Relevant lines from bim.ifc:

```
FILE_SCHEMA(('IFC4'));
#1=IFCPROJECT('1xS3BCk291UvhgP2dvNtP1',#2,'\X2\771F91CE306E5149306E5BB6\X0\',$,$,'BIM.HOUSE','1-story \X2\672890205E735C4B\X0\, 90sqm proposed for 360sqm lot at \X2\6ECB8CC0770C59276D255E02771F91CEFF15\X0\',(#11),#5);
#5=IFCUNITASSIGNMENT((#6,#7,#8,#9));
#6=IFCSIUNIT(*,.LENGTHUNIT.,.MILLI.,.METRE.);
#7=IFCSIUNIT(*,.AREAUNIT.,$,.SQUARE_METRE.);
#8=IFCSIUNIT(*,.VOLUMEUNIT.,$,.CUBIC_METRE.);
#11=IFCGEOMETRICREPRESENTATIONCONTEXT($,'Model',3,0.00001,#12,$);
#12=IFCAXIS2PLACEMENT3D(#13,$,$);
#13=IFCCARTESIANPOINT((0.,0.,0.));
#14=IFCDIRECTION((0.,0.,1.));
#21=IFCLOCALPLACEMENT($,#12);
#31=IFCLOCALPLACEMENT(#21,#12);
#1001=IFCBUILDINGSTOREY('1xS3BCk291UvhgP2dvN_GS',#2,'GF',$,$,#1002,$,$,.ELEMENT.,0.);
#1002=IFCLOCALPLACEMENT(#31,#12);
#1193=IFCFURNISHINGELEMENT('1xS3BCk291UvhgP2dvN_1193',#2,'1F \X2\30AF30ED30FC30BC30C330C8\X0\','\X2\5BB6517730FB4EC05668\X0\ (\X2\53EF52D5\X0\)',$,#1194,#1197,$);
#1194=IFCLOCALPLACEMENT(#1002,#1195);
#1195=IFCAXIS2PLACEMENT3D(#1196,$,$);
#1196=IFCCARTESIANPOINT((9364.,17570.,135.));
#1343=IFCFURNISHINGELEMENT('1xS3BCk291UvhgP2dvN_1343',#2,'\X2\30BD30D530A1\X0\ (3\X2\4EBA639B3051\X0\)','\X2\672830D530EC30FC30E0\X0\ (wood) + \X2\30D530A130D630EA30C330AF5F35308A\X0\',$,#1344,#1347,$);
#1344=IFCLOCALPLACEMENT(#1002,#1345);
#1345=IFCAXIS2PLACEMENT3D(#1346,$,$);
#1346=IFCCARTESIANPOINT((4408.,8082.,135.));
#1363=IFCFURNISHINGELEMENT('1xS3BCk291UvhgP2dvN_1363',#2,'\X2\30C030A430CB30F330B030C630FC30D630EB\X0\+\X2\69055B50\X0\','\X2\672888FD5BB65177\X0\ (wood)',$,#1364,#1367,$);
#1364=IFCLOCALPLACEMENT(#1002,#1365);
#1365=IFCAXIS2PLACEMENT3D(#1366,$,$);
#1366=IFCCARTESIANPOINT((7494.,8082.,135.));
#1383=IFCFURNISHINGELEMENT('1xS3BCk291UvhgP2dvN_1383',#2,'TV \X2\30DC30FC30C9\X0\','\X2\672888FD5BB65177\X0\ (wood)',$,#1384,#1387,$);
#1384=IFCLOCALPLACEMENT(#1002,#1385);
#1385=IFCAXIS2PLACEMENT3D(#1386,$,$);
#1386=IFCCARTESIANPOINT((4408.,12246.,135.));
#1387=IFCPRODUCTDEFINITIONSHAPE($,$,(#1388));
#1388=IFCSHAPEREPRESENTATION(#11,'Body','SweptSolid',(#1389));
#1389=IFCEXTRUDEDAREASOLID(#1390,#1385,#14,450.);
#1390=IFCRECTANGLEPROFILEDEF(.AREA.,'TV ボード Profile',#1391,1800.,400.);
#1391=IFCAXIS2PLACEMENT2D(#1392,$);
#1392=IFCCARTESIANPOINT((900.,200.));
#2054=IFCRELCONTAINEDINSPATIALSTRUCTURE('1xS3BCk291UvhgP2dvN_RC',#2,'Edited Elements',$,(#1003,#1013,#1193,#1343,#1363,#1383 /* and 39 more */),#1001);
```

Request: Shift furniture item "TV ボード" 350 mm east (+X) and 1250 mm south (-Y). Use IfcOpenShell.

```python
import ifcopenshell
import ifcopenshell.api.geometry
import ifcopenshell.util.placement
import ifcopenshell.util.unit

model = ifcopenshell.open("bim.ifc")
unit_scale = ifcopenshell.util.unit.calculate_unit_scale(model)

item = model.by_guid("1xS3BCk291UvhgP2dvN_1383")
matrix = ifcopenshell.util.placement.get_local_placement(item.ObjectPlacement)
matrix[0, 3] += 0.35 / unit_scale
matrix[1, 3] -= 1.25 / unit_scale
ifcopenshell.api.geometry.edit_object_placement(model, product=item, matrix=matrix, is_si=False)

print(ifcopenshell.util.placement.get_local_placement(item.ObjectPlacement).round(3) + 0.0)

model.write("bim_rev.ifc")
```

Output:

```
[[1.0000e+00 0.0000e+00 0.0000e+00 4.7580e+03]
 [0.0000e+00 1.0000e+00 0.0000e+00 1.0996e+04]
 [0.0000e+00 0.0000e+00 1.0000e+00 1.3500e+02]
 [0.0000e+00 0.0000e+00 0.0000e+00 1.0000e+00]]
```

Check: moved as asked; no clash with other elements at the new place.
